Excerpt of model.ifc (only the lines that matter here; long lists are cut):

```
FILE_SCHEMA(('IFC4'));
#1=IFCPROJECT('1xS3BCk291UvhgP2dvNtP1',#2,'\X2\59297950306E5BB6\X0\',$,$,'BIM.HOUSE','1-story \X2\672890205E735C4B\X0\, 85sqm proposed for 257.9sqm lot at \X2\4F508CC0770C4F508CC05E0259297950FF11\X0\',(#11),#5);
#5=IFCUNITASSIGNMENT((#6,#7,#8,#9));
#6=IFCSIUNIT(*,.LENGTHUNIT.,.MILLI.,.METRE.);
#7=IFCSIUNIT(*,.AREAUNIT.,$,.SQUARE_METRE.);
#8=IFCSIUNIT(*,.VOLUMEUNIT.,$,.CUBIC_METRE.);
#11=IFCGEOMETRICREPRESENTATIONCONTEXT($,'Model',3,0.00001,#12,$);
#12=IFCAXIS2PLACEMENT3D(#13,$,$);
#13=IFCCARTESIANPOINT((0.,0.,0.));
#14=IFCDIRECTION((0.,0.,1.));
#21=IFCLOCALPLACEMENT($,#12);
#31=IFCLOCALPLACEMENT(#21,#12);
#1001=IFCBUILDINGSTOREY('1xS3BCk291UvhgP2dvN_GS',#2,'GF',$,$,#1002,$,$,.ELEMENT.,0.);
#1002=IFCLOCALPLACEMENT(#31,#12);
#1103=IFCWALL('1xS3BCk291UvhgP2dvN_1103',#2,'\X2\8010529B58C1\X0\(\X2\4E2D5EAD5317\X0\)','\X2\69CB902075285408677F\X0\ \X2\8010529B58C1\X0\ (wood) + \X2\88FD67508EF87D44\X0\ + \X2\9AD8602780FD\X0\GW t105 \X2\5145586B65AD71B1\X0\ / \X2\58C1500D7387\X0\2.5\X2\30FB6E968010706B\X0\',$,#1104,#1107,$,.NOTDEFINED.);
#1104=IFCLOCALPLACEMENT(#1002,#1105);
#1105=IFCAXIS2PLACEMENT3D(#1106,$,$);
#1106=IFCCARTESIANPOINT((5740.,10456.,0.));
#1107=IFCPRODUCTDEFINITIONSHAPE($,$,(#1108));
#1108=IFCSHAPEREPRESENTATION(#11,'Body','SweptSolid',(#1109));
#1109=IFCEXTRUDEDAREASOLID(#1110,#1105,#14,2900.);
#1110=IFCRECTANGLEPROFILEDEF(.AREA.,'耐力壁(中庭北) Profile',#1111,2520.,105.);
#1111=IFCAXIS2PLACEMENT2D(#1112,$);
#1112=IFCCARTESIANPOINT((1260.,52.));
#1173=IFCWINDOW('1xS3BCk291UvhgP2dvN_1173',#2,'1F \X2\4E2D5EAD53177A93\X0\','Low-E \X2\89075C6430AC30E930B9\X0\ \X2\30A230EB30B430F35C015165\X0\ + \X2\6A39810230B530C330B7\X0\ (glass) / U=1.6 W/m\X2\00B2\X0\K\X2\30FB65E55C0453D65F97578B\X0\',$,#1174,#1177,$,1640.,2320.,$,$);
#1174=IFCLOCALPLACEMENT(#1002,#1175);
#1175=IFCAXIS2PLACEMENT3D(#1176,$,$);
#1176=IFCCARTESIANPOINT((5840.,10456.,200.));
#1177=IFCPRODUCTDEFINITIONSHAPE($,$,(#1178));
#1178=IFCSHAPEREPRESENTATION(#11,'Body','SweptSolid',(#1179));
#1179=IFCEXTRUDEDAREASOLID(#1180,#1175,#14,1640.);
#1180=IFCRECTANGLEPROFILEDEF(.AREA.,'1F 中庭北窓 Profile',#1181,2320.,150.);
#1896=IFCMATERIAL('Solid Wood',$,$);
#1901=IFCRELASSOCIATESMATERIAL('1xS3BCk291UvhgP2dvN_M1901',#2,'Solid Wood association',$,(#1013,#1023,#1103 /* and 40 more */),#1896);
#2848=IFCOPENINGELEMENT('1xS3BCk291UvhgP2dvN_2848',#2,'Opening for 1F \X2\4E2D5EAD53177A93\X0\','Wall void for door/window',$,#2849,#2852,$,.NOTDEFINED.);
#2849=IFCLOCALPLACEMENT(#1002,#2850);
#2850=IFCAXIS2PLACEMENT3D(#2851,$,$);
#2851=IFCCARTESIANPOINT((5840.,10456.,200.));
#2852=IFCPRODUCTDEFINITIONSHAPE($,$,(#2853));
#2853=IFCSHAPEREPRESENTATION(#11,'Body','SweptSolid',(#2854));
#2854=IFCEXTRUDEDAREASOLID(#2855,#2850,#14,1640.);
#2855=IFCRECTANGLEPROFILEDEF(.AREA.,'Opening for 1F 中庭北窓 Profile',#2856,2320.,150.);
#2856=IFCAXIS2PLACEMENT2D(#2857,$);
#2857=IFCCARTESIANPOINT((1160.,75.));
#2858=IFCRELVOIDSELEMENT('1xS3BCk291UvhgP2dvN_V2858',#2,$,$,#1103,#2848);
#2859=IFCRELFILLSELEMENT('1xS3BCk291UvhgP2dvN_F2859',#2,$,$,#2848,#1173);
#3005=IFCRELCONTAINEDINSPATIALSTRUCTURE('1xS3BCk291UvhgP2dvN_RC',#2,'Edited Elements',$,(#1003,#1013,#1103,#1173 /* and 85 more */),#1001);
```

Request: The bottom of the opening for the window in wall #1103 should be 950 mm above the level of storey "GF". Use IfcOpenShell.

```python
import numpy as np
import ifcopenshell
import ifcopenshell.api.geometry
import ifcopenshell.geom
import ifcopenshell.util.element
import ifcopenshell.util.placement
import ifcopenshell.util.shape
import ifcopenshell.util.unit

model = ifcopenshell.open("model.ifc")
unit_scale = ifcopenshell.util.unit.calculate_unit_scale(model)

window = model.by_id(1173)
opening = window.FillsVoids[0].RelatingOpeningElement
storey = ifcopenshell.util.element.get_container(window, ifc_class="IfcBuildingStorey")
level = ifcopenshell.util.placement.get_local_placement(storey.ObjectPlacement)[2, 3]

# The opening's origin need not be at the sill, so measure its lowest point.
shape = ifcopenshell.geom.create_shape(ifcopenshell.geom.settings(), opening)
bottom = ifcopenshell.util.shape.get_shape_bottom_elevation(shape, shape.geometry) / unit_scale
dz = level + 0.95 / unit_scale - bottom

shift = np.array([0.0, 0.0, dz])
# The window is not placed relative to its opening, so move both.
for product in (opening, window):
    matrix = ifcopenshell.util.placement.get_local_placement(product.ObjectPlacement)
    matrix[:3, 3] += shift
    ifcopenshell.api.geometry.edit_object_placement(model, product=product, matrix=matrix, is_si=False)

print(f"moved by {dz * unit_scale:+.3f} m")

model.write("model_edited.ifc")
```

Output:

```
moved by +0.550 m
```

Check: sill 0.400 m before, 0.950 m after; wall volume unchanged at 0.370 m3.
